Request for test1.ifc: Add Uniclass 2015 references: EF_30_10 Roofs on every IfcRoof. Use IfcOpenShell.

First a look at what the model holds.

```python
import ifcopenshell

model = ifcopenshell.open("test1.ifc")
print(model.schema)
print("classifications:", [c.Name for c in model.by_type("IfcClassification")])
for ifc_class in ("IfcDoor", "IfcRoof", "IfcStair", "IfcWall", "IfcWindow"):
    print(ifc_class, len(model.by_type(ifc_class)))
```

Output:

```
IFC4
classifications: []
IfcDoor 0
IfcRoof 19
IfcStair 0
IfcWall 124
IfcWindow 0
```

```python
import ifcopenshell
import ifcopenshell.api.classification

model = ifcopenshell.open("test1.ifc")

system = ifcopenshell.api.classification.add_classification(model, classification="Uniclass 2015")

codes = {
    "IfcRoof": ("EF_30_10", "Roofs"),
}
for ifc_class, (code, name) in codes.items():
    products = model.by_type(ifc_class)
    ifcopenshell.api.classification.add_reference(
        model, products=products, classification=system, identification=code, name=name
    )
    print(code, len(products))

model.write("test1_v2.ifc")
```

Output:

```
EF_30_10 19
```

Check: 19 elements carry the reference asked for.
